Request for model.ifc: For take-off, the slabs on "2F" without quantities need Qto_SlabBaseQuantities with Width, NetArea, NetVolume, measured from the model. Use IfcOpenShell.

First a look at what the model holds.

```python
import ifcopenshell
import ifcopenshell.util.element
import ifcopenshell.util.unit

model = ifcopenshell.open("model.ifc")
print(model.schema)
for unit_type in ("LENGTHUNIT", "AREAUNIT", "VOLUMEUNIT"):
    print(unit_type, ifcopenshell.util.unit.calculate_unit_scale(model, unit_type))
storey = next(s for s in model.by_type("IfcBuildingStorey") if s.Name == "2F")
slabs = [e for e in ifcopenshell.util.element.get_decomposition(storey) if e.is_a("IfcSlab")]
for e in sorted(slabs, key=lambda e: e.id()):
    print(e.id(), e.is_a(), e.Name, list(ifcopenshell.util.element.get_psets(e, qtos_only=True)), sep=" | ")
```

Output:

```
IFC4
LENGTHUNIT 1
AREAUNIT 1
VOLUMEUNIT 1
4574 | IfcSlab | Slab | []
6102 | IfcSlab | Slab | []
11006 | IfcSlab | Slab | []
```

```python
import ifcopenshell
import ifcopenshell.api.pset
import ifcopenshell.geom
import ifcopenshell.util.element
import ifcopenshell.util.shape
import ifcopenshell.util.unit

model = ifcopenshell.open("model.ifc")
unit_scale = ifcopenshell.util.unit.calculate_unit_scale(model)
area_scale = ifcopenshell.util.unit.calculate_unit_scale(model, "AREAUNIT")
volume_scale = ifcopenshell.util.unit.calculate_unit_scale(model, "VOLUMEUNIT")
settings = ifcopenshell.geom.settings()

storey = next(s for s in model.by_type("IfcBuildingStorey") if s.Name == "2F")
slabs = [e for e in ifcopenshell.util.element.get_decomposition(storey) if e.is_a("IfcSlab")]

for e in sorted(slabs, key=lambda e: e.id()):
    if ifcopenshell.util.element.get_psets(e, qtos_only=True, should_inherit=False):
        continue
    # Geometry comes back in metres, in the element's own axes.
    shape = ifcopenshell.geom.create_shape(settings, e)
    values = {
        "Width": ifcopenshell.util.shape.get_z(shape.geometry) / unit_scale,
        "NetArea": ifcopenshell.util.shape.get_footprint_area(shape.geometry) / area_scale,
        "NetVolume": ifcopenshell.util.shape.get_volume(shape.geometry) / volume_scale,
    }
    qto = ifcopenshell.api.pset.add_qto(model, product=e, name="Qto_SlabBaseQuantities")
    ifcopenshell.api.pset.edit_qto(model, qto=qto, properties=values)
    print(e.id(), {k: round(v, 3) for k, v in values.items()})

model.write("model_v2.ifc")
```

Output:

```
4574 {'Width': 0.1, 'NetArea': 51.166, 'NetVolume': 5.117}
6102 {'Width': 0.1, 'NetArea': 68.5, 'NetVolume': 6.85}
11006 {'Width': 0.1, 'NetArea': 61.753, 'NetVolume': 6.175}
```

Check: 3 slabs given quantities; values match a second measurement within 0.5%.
